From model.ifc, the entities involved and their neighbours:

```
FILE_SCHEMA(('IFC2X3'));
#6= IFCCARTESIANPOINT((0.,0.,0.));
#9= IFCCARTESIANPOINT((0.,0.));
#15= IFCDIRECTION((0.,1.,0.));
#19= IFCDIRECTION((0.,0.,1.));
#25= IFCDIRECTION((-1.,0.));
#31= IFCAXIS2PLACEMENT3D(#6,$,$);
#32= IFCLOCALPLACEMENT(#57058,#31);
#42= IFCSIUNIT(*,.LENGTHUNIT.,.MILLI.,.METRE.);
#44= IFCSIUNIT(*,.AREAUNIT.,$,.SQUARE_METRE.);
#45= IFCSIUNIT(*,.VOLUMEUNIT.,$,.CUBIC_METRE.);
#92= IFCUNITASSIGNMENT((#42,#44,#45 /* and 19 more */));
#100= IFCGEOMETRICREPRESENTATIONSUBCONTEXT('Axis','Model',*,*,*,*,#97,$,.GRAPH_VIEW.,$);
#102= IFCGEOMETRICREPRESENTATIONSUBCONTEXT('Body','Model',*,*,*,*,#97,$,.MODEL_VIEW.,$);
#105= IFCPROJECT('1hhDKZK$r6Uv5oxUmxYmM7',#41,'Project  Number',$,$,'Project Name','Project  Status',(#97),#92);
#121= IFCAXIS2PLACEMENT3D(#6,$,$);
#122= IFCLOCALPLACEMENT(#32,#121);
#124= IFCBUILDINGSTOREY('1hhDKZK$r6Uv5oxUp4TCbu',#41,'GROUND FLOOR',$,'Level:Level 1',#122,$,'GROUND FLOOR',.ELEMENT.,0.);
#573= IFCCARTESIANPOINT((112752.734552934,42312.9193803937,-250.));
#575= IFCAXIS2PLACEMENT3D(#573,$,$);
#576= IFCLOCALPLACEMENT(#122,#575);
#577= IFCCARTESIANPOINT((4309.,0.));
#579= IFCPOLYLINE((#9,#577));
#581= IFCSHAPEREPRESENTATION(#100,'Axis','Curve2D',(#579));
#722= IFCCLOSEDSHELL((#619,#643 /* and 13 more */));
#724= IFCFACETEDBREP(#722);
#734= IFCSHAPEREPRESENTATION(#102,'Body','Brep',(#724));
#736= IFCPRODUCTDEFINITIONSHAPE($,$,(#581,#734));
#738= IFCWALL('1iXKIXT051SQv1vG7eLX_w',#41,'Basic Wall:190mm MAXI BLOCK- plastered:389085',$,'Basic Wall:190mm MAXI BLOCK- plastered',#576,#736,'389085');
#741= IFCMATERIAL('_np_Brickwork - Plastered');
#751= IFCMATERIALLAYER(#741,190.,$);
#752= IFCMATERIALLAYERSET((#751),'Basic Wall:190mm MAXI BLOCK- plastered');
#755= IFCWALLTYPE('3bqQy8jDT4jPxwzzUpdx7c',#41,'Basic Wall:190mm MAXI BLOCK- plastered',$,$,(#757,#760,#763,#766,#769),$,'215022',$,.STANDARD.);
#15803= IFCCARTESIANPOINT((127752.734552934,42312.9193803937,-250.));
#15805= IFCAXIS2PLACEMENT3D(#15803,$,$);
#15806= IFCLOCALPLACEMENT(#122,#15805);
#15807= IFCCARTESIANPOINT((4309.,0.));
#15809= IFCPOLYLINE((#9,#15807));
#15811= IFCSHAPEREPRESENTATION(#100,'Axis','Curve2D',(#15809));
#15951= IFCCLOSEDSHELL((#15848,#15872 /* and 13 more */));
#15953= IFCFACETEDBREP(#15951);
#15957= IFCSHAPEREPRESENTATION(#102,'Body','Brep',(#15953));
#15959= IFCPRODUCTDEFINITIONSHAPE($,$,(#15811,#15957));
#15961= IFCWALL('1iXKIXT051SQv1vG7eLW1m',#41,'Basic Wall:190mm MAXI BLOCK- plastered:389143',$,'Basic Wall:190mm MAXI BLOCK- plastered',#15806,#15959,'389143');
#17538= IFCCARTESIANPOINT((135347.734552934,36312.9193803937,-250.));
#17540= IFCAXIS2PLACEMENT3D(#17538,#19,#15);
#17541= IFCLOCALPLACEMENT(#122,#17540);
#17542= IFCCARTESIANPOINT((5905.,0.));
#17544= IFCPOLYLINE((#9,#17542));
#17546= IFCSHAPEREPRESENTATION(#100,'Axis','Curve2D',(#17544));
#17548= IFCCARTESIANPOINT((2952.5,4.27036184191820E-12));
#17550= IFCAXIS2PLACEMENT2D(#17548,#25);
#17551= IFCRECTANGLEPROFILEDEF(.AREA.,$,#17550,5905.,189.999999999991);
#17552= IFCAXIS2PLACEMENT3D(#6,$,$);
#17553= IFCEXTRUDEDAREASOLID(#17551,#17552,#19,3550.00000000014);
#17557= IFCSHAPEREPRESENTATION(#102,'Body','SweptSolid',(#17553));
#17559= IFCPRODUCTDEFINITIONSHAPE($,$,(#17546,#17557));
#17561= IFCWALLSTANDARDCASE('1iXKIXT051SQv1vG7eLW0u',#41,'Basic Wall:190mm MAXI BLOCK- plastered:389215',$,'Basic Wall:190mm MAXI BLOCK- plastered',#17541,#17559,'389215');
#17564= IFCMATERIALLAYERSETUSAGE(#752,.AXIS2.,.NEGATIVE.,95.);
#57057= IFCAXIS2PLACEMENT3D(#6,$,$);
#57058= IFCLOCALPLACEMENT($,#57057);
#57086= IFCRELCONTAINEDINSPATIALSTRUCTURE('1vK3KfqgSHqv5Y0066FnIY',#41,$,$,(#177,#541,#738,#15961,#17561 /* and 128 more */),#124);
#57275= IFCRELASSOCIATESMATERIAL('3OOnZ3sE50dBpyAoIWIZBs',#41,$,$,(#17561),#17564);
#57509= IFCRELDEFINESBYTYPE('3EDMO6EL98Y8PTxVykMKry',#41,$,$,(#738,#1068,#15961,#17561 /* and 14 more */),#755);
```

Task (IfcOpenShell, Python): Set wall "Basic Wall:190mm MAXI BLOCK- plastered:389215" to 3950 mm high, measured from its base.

```python
import ifcopenshell
import ifcopenshell.geom
import ifcopenshell.util.representation
import ifcopenshell.util.shape

model = ifcopenshell.open("model.ifc")
settings = ifcopenshell.geom.settings()


def volume(element):
    """Net volume in cubic metres, openings subtracted."""
    shape = ifcopenshell.geom.create_shape(settings, element)
    return ifcopenshell.util.shape.get_volume(shape.geometry)


wall = model.by_id(17561)
before = volume(wall)

body = ifcopenshell.util.representation.get_representation(wall, "Model", "Body")
solid = body.Items[0]
old_height = solid.Depth
solid.Depth = 3950.0
after = volume(wall)

print(f"height {old_height:g} -> {solid.Depth:g}, volume {before:.3f} -> {after:.3f} m3")

model.write("model_edited.ifc")
```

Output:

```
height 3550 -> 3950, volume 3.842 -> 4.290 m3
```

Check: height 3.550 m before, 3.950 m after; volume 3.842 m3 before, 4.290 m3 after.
